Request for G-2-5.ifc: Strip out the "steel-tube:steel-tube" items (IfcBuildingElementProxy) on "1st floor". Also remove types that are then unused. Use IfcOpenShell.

First a look at what the model holds.

```python
import ifcopenshell
import ifcopenshell.util.element

model = ifcopenshell.open("G-2-5.ifc")
print(model.schema)
storey = next(s for s in model.by_type("IfcBuildingStorey") if s.Name == "1st floor")
proxies = [e for e in ifcopenshell.util.element.get_decomposition(storey) if e.is_a("IfcBuildingElementProxy")]
seen = {}
for e in proxies:
    element_type = ifcopenshell.util.element.get_type(e)
    name = element_type.Name if element_type not in (None, e) else None
    seen[name] = seen.get(name, 0) + 1
for name, count in sorted(seen.items(), key=str):
    print(count, "x", name)
```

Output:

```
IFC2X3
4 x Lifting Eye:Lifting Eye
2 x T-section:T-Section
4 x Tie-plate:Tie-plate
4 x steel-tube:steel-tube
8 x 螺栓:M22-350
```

```python
import ifcopenshell
import ifcopenshell.api.root
import ifcopenshell.util.element

model = ifcopenshell.open("G-2-5.ifc")

storey = next(s for s in model.by_type("IfcBuildingStorey") if s.Name == "1st floor")
proxies = [e for e in ifcopenshell.util.element.get_decomposition(storey) if e.is_a("IfcBuildingElementProxy")]
targets = [e for e in proxies if (t := ifcopenshell.util.element.get_type(e)) not in (None, e) and t.Name == "steel-tube:steel-tube"]
types = {ifcopenshell.util.element.get_type(e) for e in targets} - {None, *targets}

for e in targets:
    ifcopenshell.api.root.remove_product(model, product=e)
print(len(targets), "removed")

unused = [t for t in types if not ifcopenshell.util.element.get_types(t)]
for t in unused:
    ifcopenshell.api.root.remove_product(model, product=t)
print(len(unused), "unused types removed")

model.write("G-2-5_edited.ifc")
```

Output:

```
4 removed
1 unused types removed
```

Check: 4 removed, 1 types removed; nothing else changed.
